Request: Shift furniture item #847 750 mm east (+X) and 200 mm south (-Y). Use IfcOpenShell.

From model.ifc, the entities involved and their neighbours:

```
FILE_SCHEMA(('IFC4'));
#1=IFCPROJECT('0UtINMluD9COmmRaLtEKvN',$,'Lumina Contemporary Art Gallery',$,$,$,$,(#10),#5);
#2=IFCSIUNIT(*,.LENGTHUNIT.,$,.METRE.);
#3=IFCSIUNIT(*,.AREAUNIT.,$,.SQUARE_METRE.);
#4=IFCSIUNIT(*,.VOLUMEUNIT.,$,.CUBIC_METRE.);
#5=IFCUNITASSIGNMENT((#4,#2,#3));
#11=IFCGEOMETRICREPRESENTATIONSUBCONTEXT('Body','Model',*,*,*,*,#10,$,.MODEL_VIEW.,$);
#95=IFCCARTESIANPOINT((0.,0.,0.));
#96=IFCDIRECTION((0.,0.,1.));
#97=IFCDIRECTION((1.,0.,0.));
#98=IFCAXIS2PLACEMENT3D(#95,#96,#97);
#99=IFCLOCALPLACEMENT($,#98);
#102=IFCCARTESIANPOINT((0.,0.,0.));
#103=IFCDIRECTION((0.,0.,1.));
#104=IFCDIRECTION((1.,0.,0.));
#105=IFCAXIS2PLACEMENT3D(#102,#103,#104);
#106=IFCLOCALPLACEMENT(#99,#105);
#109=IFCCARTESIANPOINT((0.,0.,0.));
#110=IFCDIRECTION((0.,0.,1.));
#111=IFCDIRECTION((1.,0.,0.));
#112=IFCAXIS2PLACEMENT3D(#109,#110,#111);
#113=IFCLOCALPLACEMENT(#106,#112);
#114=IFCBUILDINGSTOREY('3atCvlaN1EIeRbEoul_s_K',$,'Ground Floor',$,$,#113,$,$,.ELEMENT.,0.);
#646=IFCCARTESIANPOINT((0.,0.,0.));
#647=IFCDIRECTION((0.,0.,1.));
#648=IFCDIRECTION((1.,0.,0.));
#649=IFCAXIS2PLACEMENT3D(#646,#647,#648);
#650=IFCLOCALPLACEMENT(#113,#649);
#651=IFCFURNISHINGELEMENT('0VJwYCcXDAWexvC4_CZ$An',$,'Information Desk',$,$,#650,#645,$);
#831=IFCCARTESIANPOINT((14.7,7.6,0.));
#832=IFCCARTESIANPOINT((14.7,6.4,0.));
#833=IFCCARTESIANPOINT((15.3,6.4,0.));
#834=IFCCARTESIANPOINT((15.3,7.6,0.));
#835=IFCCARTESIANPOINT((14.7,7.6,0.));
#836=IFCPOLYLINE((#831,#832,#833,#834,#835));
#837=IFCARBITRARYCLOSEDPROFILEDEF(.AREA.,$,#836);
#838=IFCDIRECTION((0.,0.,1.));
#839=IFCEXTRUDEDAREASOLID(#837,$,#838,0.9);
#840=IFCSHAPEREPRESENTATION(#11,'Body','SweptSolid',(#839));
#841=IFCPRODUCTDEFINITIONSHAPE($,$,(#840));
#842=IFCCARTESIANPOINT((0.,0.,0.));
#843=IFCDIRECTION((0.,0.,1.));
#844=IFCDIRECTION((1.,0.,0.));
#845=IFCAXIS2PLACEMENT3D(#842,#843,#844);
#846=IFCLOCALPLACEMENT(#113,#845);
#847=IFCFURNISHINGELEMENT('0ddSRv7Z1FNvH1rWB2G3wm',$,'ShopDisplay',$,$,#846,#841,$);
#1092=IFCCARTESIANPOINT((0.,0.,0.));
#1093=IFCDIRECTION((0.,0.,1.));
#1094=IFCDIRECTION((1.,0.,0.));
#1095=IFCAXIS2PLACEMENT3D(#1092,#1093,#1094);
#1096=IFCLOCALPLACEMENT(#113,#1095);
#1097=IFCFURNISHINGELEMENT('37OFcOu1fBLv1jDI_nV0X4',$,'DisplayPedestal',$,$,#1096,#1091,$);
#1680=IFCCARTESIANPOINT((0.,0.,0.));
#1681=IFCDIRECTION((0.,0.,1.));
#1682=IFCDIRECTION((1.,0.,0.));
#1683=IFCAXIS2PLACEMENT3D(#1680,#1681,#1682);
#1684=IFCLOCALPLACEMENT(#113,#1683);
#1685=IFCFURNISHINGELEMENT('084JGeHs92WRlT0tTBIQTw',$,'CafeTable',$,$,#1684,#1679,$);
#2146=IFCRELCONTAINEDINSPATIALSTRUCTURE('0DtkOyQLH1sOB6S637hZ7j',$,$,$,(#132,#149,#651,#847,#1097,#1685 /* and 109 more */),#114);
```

```python
import ifcopenshell
import ifcopenshell.api.geometry
import ifcopenshell.util.placement
import ifcopenshell.util.unit

model = ifcopenshell.open("model.ifc")
unit_scale = ifcopenshell.util.unit.calculate_unit_scale(model)

item = model.by_guid("0ddSRv7Z1FNvH1rWB2G3wm")
matrix = ifcopenshell.util.placement.get_local_placement(item.ObjectPlacement)
matrix[0, 3] += 0.75 / unit_scale
matrix[1, 3] -= 0.2 / unit_scale
ifcopenshell.api.geometry.edit_object_placement(model, product=item, matrix=matrix, is_si=False)

print(ifcopenshell.util.placement.get_local_placement(item.ObjectPlacement).round(3) + 0.0)

model.write("model_v2.ifc")
```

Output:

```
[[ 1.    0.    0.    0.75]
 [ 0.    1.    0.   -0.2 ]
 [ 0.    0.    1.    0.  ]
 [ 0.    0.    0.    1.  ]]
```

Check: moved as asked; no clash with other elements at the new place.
